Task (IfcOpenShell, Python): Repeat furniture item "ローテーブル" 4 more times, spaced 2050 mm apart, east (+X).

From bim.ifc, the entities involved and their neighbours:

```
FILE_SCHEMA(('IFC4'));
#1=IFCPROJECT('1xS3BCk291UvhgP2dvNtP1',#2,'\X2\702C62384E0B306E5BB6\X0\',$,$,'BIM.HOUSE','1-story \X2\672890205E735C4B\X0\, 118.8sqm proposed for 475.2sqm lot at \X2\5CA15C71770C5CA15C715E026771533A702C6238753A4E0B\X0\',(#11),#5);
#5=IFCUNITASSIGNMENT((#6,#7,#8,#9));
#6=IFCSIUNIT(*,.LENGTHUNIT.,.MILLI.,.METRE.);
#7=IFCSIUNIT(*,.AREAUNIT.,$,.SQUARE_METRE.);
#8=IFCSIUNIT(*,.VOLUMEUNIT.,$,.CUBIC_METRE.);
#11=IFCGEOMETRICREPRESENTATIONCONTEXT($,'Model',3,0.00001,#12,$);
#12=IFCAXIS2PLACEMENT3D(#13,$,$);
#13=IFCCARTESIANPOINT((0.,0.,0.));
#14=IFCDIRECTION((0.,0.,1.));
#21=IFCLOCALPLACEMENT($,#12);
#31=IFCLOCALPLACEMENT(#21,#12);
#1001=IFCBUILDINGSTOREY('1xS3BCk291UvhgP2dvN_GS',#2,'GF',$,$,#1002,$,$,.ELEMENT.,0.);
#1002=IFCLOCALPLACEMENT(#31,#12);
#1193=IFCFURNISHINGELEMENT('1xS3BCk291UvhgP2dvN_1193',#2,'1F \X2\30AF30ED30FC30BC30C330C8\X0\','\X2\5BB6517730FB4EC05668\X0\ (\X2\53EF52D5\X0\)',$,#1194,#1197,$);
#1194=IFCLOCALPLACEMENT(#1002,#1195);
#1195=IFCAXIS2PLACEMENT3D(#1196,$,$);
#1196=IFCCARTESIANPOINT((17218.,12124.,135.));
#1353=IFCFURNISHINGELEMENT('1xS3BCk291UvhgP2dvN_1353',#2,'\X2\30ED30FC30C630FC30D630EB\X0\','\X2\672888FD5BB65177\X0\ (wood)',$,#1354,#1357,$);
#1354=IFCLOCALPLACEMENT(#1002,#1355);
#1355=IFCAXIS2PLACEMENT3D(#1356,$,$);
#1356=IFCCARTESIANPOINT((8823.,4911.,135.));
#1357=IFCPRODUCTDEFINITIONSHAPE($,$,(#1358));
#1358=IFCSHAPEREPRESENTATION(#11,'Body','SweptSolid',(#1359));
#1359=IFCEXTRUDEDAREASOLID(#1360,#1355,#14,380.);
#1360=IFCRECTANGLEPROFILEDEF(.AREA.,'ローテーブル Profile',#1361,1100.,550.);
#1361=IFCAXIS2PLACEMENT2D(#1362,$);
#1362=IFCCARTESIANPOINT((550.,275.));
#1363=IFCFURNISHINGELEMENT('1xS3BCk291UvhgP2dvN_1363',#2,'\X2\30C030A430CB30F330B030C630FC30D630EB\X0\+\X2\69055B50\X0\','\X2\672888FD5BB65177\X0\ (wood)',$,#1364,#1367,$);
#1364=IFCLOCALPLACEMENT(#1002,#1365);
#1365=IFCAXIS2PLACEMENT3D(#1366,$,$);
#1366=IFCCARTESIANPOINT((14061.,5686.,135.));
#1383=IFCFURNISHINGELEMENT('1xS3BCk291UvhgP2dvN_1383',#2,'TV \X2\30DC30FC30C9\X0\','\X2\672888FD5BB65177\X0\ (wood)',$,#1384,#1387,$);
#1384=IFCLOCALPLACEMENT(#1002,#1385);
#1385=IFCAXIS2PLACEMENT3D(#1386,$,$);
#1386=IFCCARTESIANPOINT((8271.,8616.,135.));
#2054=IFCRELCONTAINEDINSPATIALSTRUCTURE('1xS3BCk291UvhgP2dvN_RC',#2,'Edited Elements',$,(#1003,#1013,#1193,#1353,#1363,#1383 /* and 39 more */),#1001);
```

```python
import numpy as np
import ifcopenshell
import ifcopenshell.api.geometry
import ifcopenshell.api.root
import ifcopenshell.util.element
import ifcopenshell.util.placement

model = ifcopenshell.open("bim.ifc")


def reuse_history(source, copy):
    """copy_class also copies each property set's owner history, people and application; keep the originals."""
    for rel in copy.IsDefinedBy:
        if rel.is_a("IfcRelDefinesByProperties") and (history := rel.RelatingPropertyDefinition.OwnerHistory):
            rel.RelatingPropertyDefinition.OwnerHistory = source.OwnerHistory
            ifcopenshell.util.element.remove_deep2(model, history)


source = model.by_guid("1xS3BCk291UvhgP2dvN_1353")
base = ifcopenshell.util.placement.get_local_placement(source.ObjectPlacement)
step = np.array([1.0, 0.0, 0.0]) * 2050.0

for i in range(1, 5):
    copy = ifcopenshell.api.root.copy_class(model, product=source)
    copy.Representation = ifcopenshell.util.element.copy_deep(
        model, source.Representation, exclude=["IfcGeometricRepresentationContext", "IfcRepresentationMap"]
    )
    reuse_history(source, copy)
    matrix = base.copy()
    matrix[:3, 3] += i * step
    print("added at", matrix[:3, 3].round(3) + 0.0)
    ifcopenshell.api.geometry.edit_object_placement(model, product=copy, matrix=matrix, is_si=False)

model.write("bim_v2.ifc")
```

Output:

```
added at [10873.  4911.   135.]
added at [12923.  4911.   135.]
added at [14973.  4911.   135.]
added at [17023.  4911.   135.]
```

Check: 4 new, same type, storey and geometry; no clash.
